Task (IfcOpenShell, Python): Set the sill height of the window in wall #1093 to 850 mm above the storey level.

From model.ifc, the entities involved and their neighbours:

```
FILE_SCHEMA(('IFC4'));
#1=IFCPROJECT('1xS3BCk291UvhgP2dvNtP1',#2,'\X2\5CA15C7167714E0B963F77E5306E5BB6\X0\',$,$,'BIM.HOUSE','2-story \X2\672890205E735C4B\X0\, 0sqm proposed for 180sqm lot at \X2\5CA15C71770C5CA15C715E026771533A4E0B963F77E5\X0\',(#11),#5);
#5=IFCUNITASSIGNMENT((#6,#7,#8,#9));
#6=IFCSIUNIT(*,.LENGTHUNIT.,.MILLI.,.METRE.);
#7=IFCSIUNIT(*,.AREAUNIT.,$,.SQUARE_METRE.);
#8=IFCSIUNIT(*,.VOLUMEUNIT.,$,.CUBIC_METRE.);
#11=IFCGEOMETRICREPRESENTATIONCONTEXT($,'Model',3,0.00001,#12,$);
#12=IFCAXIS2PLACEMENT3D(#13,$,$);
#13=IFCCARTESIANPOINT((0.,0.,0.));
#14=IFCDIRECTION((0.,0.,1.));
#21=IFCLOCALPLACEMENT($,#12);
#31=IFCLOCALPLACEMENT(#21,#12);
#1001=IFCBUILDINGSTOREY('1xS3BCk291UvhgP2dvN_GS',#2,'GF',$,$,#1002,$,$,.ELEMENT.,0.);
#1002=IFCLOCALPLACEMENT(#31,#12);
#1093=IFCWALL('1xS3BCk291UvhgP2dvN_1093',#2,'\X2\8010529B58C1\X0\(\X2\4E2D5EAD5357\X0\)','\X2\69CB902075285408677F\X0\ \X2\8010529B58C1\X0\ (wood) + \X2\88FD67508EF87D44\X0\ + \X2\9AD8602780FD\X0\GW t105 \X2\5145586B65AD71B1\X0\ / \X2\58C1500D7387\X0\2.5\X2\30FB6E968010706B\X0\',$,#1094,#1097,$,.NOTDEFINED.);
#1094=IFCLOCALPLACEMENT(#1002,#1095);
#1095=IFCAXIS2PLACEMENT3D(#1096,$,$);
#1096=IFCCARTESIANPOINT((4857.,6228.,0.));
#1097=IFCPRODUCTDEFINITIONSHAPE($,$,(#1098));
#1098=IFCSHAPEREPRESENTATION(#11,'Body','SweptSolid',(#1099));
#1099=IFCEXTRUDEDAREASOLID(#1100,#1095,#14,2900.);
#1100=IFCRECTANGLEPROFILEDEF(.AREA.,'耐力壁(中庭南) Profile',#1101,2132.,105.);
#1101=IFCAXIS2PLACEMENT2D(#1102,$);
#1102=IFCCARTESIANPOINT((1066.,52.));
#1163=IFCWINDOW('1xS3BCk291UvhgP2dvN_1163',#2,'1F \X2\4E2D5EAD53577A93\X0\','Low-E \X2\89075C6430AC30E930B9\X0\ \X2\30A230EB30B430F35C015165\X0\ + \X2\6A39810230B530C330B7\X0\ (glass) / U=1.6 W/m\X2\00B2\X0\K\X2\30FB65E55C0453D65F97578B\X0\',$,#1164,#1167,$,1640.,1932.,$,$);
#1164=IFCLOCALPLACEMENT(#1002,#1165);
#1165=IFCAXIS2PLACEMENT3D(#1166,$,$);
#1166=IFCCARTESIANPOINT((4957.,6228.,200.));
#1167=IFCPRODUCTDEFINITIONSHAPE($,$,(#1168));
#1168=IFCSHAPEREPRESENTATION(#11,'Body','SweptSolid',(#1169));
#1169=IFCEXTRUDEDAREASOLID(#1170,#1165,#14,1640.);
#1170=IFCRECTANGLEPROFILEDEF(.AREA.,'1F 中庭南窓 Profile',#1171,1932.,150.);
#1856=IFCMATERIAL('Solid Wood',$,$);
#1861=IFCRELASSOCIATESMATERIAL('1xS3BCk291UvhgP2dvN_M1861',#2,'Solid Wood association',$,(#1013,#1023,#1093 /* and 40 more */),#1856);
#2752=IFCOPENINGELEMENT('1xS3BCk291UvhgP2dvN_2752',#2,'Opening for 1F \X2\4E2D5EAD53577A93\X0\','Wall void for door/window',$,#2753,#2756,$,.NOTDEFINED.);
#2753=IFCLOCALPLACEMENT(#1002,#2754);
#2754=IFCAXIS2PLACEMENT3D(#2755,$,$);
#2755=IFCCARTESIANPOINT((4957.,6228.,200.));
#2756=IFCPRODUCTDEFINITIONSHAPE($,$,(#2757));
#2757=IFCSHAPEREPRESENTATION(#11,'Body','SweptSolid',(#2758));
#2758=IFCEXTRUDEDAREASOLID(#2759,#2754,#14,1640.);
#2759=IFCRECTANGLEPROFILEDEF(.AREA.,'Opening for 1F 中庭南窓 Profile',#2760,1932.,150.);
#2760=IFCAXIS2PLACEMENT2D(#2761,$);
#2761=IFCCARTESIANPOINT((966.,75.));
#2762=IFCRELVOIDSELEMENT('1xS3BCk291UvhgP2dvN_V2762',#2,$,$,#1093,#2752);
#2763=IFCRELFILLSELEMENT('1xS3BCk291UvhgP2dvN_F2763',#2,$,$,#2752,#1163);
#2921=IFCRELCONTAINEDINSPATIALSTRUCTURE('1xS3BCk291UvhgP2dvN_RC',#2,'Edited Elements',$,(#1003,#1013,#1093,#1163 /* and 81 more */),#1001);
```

```python
import numpy as np
import ifcopenshell
import ifcopenshell.api.geometry
import ifcopenshell.geom
import ifcopenshell.util.element
import ifcopenshell.util.placement
import ifcopenshell.util.shape
import ifcopenshell.util.unit

model = ifcopenshell.open("model.ifc")
unit_scale = ifcopenshell.util.unit.calculate_unit_scale(model)

window = model.by_id(1163)
opening = window.FillsVoids[0].RelatingOpeningElement
storey = ifcopenshell.util.element.get_container(window, ifc_class="IfcBuildingStorey")
level = ifcopenshell.util.placement.get_local_placement(storey.ObjectPlacement)[2, 3]

# The opening's origin need not be at the sill, so measure its lowest point.
shape = ifcopenshell.geom.create_shape(ifcopenshell.geom.settings(), opening)
bottom = ifcopenshell.util.shape.get_shape_bottom_elevation(shape, shape.geometry) / unit_scale
dz = level + 0.85 / unit_scale - bottom

shift = np.array([0.0, 0.0, dz])
# The window is not placed relative to its opening, so move both.
for product in (opening, window):
    matrix = ifcopenshell.util.placement.get_local_placement(product.ObjectPlacement)
    matrix[:3, 3] += shift
    ifcopenshell.api.geometry.edit_object_placement(model, product=product, matrix=matrix, is_si=False)

print(f"moved by {dz * unit_scale:+.3f} m")

model.write("model_edited.ifc")
```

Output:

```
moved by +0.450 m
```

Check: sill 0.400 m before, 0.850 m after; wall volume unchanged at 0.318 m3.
